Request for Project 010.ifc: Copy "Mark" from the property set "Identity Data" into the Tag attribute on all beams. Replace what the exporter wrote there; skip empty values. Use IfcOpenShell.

First a look at what the model holds.

```python
import ifcopenshell
import ifcopenshell.util.element

model = ifcopenshell.open("Project 010.ifc")
print(model.schema)
beams = model.by_type("IfcBeam")
print(len(beams), "beams")
for e in beams[:8]:
    source = ifcopenshell.util.element.get_pset(e, "Identity Data", "Mark")
    target = e.Tag
    print(e.id(), repr(source), repr(target), sep=" | ")
```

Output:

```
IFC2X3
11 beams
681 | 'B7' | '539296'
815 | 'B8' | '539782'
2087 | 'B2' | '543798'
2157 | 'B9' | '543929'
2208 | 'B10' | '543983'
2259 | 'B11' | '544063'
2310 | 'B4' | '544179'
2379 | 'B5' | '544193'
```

```python
import ifcopenshell
import ifcopenshell.util.element

model = ifcopenshell.open("Project 010.ifc")

count = 0
for e in model.by_type("IfcBeam"):
    value = ifcopenshell.util.element.get_pset(e, "Identity Data", "Mark")
    current = e.Tag
    if not value or not value.strip() or current == value:
        continue
    e.Tag = value
    count += 1

print(count, "beams updated")

model.write("Project 010_updated.ifc")
```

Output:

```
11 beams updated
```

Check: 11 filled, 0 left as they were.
